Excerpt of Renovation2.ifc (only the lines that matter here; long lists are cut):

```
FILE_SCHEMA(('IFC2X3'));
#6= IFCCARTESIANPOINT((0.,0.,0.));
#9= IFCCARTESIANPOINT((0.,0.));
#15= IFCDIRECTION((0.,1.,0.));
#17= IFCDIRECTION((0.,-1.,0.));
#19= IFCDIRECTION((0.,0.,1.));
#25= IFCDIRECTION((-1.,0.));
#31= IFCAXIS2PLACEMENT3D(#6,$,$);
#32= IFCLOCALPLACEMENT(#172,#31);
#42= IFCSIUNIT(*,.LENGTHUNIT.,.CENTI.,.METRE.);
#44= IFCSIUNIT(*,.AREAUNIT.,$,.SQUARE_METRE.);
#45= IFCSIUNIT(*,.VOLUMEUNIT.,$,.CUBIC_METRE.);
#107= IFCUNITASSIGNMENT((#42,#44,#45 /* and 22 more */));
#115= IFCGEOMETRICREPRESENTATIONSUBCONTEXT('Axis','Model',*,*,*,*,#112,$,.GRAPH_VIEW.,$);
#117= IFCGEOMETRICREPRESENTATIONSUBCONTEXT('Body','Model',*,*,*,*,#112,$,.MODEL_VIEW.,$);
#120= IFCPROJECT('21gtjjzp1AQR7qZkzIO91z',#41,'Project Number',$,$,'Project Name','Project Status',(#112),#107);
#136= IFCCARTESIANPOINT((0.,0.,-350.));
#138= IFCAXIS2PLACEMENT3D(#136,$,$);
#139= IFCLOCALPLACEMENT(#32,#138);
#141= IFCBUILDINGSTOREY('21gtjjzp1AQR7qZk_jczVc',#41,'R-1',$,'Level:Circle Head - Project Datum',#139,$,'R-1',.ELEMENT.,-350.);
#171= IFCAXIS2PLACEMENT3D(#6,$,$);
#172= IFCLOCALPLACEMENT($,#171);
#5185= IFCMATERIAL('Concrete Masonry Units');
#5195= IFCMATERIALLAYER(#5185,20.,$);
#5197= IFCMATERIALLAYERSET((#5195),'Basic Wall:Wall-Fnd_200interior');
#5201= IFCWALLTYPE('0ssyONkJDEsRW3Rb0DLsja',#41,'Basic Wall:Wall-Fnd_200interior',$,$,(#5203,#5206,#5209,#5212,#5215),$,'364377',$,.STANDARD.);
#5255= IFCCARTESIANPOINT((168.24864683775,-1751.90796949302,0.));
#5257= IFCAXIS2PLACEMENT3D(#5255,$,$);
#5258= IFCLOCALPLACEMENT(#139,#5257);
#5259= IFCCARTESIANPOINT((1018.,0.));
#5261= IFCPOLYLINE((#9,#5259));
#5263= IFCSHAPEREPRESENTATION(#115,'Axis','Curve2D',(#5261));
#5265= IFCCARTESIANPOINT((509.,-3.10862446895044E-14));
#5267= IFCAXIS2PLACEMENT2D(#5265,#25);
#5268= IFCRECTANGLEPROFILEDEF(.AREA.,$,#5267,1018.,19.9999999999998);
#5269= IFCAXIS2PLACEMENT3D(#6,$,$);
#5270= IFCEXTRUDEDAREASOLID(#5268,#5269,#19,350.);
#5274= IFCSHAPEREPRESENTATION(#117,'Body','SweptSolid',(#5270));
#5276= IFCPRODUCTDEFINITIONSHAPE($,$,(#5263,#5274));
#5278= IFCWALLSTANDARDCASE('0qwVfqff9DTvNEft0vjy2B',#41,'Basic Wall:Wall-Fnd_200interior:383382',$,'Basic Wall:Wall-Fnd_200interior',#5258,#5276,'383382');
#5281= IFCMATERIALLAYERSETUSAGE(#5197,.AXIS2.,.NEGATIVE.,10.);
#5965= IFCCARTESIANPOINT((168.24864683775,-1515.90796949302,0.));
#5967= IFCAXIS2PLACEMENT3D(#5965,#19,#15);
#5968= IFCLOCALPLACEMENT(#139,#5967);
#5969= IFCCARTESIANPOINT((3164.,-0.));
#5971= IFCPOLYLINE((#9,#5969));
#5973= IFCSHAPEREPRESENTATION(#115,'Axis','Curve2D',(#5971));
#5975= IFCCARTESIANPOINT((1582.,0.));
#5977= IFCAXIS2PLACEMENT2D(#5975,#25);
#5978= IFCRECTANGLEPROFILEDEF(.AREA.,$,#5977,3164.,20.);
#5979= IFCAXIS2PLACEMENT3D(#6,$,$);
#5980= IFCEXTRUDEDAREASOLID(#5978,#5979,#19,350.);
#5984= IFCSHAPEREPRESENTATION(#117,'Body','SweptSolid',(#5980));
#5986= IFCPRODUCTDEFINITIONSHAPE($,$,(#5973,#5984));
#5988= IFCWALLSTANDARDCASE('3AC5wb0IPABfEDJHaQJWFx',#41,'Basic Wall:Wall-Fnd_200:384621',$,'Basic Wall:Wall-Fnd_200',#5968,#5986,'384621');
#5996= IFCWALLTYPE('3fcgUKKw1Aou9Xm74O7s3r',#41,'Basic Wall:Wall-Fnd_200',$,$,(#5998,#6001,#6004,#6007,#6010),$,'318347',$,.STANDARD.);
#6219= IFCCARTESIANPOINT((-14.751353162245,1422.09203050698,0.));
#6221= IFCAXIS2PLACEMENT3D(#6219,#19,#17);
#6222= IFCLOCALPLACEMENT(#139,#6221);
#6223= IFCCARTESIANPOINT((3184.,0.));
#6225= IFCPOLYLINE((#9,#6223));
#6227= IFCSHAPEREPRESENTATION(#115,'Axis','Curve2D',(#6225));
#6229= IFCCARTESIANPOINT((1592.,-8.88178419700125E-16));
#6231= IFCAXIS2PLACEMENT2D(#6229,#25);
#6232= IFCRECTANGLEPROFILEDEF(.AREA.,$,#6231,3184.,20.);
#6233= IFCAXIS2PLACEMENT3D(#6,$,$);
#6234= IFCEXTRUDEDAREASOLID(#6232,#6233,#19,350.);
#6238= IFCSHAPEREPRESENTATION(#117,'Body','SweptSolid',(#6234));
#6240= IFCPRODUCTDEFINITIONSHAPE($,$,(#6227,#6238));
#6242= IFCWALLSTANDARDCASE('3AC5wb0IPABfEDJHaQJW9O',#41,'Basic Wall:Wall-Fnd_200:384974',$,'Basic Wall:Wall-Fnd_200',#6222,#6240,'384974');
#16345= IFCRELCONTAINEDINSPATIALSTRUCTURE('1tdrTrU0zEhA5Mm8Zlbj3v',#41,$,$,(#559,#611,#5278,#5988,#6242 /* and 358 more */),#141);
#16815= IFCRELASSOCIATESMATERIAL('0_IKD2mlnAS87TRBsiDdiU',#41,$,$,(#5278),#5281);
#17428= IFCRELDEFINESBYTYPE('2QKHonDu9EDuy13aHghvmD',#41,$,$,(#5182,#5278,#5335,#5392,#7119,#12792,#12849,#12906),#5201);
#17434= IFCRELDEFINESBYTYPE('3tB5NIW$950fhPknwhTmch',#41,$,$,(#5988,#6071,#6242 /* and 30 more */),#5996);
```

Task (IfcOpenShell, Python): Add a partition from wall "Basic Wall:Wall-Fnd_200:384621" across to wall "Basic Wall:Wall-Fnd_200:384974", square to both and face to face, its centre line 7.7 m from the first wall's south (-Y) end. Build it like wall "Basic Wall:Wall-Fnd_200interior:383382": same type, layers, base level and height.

```python
import numpy as np
import ifcopenshell
import ifcopenshell.api.geometry
import ifcopenshell.api.material
import ifcopenshell.api.pset
import ifcopenshell.api.root
import ifcopenshell.api.spatial
import ifcopenshell.api.type
import ifcopenshell.geom
import ifcopenshell.util.element
import ifcopenshell.util.placement
import ifcopenshell.util.representation
import ifcopenshell.util.shape
import ifcopenshell.util.unit

model = ifcopenshell.open("Renovation2.ifc")
unit_scale = ifcopenshell.util.unit.calculate_unit_scale(model)
settings = ifcopenshell.geom.settings()
settings.set("use-world-coords", True)

start_wall = model.by_id(5988)
end_wall = model.by_id(6242)
like = model.by_guid("0qwVfqff9DTvNEft0vjy2B")
matrix = ifcopenshell.util.placement.get_local_placement(start_wall.ObjectPlacement)
matrix[:3, 3] *= unit_scale


def extent(element):
    """Bounding box in the first wall's axes, in metres."""
    shape = ifcopenshell.geom.create_shape(settings, element)
    points = (ifcopenshell.util.shape.get_vertices(shape.geometry) - matrix[:3, 3]) @ matrix[:3, :3]
    return points.min(axis=0), points.max(axis=0)


y_start = extent(start_wall)[1][1]
y_end = extent(end_wall)[0][1]
like_min, like_max = extent(like)
length, height = float(abs(y_end - y_start)), float(like_max[2] - like_min[2])
layer_set = ifcopenshell.util.element.get_material(like, should_skip_usage=True)
thickness = sum(layer.LayerThickness for layer in layer_set.MaterialLayers) * unit_scale

wall = ifcopenshell.api.root.create_entity(model, ifc_class="IfcWallStandardCase", name="New partition")
storey = ifcopenshell.util.element.get_container(like)
ifcopenshell.api.spatial.assign_container(model, products=[wall], relating_structure=storey)
ifcopenshell.api.type.assign_type(
    model, related_objects=[wall], relating_type=ifcopenshell.util.element.get_type(like), should_map_representations=False
)
rel = ifcopenshell.api.material.assign_material(
    model, products=[wall], type="IfcMaterialLayerSetUsage", material=layer_set
)
rel.RelatingMaterial.OffsetFromReferenceLine = -thickness / 2 / unit_scale
pset = ifcopenshell.api.pset.add_pset(model, product=wall, name="Pset_WallCommon")
ifcopenshell.api.pset.edit_pset(model, pset=pset, properties={"IsExternal": False, "LoadBearing": False})

# The axis runs down the middle of the wall.
axis = ifcopenshell.api.geometry.add_axis_representation(
    model, context=ifcopenshell.util.representation.get_context(model, "Model", "Axis"), axis=[(0.0, 0.0), (length, 0.0)]
)
body = ifcopenshell.api.geometry.add_wall_representation(
    model,
    context=ifcopenshell.util.representation.get_context(model, "Model", "Body", "MODEL_VIEW"),
    length=length,
    height=height,
    thickness=thickness,
    offset=-thickness / 2,
)
for representation in (axis, body):
    ifcopenshell.api.geometry.assign_representation(model, product=wall, representation=representation)

placement = matrix @ ifcopenshell.util.placement.rotation(90, "Z")
placement[:, 3] = matrix @ np.array([extent(start_wall)[0][0] + 7.7, y_start, like_min[2], 1.0])
ifcopenshell.api.geometry.edit_object_placement(model, product=wall, matrix=placement)

print(f"partition {length:.3f} m long, {height:.3f} m high, {thickness:.3f} m thick")

model.write("Renovation2_rev.ifc")
```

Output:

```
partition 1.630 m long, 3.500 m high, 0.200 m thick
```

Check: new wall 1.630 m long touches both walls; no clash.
